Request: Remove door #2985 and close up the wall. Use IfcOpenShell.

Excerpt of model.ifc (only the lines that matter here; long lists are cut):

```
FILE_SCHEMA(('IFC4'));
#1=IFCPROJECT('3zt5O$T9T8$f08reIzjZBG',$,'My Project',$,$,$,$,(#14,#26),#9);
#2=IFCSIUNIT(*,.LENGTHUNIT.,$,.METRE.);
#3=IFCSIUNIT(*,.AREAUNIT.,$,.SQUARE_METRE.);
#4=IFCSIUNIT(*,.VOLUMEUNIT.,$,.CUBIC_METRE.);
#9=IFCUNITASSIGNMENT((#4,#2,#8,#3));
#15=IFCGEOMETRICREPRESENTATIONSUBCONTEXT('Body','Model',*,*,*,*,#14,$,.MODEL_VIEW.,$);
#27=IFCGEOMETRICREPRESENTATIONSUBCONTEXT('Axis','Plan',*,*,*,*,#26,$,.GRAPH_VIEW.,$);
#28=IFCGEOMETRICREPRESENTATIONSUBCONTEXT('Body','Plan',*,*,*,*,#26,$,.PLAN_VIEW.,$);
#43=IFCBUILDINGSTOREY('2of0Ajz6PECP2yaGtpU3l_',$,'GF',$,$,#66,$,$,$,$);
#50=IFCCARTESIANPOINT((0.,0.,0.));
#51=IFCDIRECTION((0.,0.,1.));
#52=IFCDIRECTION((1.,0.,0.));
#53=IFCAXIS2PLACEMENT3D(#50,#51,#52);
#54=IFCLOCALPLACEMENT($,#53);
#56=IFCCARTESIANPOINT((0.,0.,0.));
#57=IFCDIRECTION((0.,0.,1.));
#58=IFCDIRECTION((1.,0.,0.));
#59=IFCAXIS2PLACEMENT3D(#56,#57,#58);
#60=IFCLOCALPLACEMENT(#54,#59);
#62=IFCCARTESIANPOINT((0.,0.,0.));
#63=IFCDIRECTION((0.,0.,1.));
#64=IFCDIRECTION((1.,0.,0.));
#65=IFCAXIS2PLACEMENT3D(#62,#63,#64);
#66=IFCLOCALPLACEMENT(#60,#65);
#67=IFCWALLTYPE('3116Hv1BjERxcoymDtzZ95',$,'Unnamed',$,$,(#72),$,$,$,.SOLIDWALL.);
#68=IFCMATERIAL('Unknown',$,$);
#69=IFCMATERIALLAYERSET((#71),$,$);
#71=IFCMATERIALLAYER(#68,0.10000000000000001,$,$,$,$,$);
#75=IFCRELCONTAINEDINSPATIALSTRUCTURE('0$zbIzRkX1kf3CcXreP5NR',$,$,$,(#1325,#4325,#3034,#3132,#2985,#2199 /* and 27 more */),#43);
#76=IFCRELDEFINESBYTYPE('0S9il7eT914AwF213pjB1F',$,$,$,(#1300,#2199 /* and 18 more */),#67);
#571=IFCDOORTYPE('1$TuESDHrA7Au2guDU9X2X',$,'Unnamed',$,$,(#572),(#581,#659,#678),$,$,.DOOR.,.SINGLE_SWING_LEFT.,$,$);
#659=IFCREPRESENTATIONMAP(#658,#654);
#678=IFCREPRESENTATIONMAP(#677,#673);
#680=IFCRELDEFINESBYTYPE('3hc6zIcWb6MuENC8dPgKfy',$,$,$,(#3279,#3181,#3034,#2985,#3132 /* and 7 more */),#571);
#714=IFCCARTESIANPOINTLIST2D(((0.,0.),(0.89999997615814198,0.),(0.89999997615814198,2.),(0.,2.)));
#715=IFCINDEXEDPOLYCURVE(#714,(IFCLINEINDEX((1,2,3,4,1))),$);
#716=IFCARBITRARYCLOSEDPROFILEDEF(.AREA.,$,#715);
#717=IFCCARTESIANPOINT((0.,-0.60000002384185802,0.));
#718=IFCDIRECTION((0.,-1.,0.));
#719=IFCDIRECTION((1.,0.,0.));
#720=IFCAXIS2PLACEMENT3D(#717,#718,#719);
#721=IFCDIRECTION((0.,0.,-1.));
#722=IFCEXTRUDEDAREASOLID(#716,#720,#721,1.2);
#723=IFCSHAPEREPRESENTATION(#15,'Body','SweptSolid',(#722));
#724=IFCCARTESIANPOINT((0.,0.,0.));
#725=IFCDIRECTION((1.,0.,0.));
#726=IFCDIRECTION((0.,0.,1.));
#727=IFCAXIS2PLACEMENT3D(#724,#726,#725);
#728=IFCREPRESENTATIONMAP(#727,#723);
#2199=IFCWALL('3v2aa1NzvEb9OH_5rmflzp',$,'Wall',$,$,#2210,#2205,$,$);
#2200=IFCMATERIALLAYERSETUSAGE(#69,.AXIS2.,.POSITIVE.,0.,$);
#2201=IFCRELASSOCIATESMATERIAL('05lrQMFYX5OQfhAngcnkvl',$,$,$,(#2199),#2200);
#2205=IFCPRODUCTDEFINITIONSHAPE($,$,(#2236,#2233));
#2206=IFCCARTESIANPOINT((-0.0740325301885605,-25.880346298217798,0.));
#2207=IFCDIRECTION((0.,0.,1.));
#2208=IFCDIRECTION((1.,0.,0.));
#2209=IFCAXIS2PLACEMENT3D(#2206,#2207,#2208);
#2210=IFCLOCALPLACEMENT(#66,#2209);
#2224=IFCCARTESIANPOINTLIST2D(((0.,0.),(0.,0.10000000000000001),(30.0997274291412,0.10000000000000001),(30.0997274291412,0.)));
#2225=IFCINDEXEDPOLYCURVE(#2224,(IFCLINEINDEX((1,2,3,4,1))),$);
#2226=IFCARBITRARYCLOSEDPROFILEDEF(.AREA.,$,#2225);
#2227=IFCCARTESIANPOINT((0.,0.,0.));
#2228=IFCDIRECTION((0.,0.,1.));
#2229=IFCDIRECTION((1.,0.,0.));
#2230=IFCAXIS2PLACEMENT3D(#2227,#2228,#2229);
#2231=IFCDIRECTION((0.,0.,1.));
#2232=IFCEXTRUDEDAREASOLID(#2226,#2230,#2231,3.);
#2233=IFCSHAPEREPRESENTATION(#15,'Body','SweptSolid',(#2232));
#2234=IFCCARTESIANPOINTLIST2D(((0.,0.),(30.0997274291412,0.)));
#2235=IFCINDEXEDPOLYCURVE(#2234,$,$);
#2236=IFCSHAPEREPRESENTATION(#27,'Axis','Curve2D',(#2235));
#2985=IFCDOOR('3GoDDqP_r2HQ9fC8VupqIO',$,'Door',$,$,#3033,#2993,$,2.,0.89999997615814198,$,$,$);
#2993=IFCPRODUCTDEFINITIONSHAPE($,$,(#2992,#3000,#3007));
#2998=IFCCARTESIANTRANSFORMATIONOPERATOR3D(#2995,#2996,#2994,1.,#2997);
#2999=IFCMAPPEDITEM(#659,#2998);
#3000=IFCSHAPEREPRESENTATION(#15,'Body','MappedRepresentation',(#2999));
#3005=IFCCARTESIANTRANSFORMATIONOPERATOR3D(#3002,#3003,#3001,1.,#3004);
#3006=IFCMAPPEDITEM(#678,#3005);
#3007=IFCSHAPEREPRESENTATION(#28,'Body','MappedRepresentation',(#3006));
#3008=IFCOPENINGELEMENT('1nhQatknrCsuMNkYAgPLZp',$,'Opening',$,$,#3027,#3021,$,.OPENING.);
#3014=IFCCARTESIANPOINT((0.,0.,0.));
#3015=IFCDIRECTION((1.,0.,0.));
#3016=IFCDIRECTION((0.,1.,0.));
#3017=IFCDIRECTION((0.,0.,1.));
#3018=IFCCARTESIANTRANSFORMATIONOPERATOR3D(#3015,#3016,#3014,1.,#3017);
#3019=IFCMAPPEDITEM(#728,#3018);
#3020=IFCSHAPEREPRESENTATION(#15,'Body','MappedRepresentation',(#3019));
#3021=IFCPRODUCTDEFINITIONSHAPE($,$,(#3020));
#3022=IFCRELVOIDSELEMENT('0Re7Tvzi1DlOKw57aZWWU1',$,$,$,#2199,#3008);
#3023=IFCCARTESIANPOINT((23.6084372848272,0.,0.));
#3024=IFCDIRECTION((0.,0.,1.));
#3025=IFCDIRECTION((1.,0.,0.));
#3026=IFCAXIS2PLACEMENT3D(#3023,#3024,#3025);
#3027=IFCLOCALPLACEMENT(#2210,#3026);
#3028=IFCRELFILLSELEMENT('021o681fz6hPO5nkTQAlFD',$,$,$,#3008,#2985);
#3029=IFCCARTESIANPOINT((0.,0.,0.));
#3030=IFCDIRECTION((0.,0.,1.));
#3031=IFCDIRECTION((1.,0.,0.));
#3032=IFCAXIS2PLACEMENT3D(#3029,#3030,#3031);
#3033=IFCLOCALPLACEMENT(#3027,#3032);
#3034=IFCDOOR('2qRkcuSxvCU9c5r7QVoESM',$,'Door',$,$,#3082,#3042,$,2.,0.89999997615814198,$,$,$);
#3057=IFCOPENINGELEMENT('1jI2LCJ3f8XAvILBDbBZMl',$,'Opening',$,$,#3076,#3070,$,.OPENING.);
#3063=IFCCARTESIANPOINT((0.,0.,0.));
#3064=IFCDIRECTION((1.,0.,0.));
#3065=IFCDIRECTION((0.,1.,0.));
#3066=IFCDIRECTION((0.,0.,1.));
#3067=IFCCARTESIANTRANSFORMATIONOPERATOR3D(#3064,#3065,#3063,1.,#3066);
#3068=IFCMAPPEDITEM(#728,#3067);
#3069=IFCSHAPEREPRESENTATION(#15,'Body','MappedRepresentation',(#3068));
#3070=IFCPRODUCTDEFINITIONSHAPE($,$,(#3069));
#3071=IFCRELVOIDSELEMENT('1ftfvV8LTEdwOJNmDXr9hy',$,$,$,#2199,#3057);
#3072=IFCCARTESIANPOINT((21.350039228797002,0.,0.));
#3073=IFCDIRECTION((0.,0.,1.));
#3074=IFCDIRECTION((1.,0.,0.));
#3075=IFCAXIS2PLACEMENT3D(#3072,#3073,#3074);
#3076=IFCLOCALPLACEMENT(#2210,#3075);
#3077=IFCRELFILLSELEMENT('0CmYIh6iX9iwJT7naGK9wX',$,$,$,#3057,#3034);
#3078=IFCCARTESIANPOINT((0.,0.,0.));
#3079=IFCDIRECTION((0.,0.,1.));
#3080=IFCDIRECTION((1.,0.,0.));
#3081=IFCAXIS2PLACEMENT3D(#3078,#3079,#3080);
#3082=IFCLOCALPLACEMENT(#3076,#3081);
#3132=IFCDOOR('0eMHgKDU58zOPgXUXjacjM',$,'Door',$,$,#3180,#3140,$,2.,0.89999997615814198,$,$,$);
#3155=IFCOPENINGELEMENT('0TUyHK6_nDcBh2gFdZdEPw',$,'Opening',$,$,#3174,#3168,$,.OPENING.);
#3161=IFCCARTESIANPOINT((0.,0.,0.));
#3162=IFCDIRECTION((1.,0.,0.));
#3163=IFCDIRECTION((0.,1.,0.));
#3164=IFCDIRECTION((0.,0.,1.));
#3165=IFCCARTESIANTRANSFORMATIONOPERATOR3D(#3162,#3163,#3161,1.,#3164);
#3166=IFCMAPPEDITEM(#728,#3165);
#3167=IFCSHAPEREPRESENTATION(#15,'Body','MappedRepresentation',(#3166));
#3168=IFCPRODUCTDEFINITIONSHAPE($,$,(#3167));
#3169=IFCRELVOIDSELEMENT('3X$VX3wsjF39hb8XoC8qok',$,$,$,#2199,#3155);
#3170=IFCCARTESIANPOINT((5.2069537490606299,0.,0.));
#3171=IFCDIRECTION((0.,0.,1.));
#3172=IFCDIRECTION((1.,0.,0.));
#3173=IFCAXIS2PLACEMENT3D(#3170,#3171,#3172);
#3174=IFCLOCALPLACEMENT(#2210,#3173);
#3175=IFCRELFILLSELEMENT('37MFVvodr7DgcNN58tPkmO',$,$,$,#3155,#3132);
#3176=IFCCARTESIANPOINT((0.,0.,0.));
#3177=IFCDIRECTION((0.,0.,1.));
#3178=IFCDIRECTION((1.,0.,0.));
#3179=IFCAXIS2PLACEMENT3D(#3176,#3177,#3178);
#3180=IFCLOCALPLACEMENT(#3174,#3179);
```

```python
import ifcopenshell
import ifcopenshell.api.feature
import ifcopenshell.api.root
import ifcopenshell.geom
import ifcopenshell.util.shape

model = ifcopenshell.open("model.ifc")
settings = ifcopenshell.geom.settings()


def volume(element):
    """Net volume in cubic metres, openings subtracted."""
    shape = ifcopenshell.geom.create_shape(settings, element)
    return ifcopenshell.util.shape.get_volume(shape.geometry)


door = model.by_guid("3GoDDqP_r2HQ9fC8VupqIO")
opening = door.FillsVoids[0].RelatingOpeningElement
wall = opening.VoidsElements[0].RelatingBuildingElement
before = volume(wall)

ifcopenshell.api.root.remove_product(model, product=door)
ifcopenshell.api.feature.remove_feature(model, feature=opening)

after = volume(wall)

print(f"wall volume {before:.3f} -> {after:.3f} m3")

model.write("model_v2.ifc")
```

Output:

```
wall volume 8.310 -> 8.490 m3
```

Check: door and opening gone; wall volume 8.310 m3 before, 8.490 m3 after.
